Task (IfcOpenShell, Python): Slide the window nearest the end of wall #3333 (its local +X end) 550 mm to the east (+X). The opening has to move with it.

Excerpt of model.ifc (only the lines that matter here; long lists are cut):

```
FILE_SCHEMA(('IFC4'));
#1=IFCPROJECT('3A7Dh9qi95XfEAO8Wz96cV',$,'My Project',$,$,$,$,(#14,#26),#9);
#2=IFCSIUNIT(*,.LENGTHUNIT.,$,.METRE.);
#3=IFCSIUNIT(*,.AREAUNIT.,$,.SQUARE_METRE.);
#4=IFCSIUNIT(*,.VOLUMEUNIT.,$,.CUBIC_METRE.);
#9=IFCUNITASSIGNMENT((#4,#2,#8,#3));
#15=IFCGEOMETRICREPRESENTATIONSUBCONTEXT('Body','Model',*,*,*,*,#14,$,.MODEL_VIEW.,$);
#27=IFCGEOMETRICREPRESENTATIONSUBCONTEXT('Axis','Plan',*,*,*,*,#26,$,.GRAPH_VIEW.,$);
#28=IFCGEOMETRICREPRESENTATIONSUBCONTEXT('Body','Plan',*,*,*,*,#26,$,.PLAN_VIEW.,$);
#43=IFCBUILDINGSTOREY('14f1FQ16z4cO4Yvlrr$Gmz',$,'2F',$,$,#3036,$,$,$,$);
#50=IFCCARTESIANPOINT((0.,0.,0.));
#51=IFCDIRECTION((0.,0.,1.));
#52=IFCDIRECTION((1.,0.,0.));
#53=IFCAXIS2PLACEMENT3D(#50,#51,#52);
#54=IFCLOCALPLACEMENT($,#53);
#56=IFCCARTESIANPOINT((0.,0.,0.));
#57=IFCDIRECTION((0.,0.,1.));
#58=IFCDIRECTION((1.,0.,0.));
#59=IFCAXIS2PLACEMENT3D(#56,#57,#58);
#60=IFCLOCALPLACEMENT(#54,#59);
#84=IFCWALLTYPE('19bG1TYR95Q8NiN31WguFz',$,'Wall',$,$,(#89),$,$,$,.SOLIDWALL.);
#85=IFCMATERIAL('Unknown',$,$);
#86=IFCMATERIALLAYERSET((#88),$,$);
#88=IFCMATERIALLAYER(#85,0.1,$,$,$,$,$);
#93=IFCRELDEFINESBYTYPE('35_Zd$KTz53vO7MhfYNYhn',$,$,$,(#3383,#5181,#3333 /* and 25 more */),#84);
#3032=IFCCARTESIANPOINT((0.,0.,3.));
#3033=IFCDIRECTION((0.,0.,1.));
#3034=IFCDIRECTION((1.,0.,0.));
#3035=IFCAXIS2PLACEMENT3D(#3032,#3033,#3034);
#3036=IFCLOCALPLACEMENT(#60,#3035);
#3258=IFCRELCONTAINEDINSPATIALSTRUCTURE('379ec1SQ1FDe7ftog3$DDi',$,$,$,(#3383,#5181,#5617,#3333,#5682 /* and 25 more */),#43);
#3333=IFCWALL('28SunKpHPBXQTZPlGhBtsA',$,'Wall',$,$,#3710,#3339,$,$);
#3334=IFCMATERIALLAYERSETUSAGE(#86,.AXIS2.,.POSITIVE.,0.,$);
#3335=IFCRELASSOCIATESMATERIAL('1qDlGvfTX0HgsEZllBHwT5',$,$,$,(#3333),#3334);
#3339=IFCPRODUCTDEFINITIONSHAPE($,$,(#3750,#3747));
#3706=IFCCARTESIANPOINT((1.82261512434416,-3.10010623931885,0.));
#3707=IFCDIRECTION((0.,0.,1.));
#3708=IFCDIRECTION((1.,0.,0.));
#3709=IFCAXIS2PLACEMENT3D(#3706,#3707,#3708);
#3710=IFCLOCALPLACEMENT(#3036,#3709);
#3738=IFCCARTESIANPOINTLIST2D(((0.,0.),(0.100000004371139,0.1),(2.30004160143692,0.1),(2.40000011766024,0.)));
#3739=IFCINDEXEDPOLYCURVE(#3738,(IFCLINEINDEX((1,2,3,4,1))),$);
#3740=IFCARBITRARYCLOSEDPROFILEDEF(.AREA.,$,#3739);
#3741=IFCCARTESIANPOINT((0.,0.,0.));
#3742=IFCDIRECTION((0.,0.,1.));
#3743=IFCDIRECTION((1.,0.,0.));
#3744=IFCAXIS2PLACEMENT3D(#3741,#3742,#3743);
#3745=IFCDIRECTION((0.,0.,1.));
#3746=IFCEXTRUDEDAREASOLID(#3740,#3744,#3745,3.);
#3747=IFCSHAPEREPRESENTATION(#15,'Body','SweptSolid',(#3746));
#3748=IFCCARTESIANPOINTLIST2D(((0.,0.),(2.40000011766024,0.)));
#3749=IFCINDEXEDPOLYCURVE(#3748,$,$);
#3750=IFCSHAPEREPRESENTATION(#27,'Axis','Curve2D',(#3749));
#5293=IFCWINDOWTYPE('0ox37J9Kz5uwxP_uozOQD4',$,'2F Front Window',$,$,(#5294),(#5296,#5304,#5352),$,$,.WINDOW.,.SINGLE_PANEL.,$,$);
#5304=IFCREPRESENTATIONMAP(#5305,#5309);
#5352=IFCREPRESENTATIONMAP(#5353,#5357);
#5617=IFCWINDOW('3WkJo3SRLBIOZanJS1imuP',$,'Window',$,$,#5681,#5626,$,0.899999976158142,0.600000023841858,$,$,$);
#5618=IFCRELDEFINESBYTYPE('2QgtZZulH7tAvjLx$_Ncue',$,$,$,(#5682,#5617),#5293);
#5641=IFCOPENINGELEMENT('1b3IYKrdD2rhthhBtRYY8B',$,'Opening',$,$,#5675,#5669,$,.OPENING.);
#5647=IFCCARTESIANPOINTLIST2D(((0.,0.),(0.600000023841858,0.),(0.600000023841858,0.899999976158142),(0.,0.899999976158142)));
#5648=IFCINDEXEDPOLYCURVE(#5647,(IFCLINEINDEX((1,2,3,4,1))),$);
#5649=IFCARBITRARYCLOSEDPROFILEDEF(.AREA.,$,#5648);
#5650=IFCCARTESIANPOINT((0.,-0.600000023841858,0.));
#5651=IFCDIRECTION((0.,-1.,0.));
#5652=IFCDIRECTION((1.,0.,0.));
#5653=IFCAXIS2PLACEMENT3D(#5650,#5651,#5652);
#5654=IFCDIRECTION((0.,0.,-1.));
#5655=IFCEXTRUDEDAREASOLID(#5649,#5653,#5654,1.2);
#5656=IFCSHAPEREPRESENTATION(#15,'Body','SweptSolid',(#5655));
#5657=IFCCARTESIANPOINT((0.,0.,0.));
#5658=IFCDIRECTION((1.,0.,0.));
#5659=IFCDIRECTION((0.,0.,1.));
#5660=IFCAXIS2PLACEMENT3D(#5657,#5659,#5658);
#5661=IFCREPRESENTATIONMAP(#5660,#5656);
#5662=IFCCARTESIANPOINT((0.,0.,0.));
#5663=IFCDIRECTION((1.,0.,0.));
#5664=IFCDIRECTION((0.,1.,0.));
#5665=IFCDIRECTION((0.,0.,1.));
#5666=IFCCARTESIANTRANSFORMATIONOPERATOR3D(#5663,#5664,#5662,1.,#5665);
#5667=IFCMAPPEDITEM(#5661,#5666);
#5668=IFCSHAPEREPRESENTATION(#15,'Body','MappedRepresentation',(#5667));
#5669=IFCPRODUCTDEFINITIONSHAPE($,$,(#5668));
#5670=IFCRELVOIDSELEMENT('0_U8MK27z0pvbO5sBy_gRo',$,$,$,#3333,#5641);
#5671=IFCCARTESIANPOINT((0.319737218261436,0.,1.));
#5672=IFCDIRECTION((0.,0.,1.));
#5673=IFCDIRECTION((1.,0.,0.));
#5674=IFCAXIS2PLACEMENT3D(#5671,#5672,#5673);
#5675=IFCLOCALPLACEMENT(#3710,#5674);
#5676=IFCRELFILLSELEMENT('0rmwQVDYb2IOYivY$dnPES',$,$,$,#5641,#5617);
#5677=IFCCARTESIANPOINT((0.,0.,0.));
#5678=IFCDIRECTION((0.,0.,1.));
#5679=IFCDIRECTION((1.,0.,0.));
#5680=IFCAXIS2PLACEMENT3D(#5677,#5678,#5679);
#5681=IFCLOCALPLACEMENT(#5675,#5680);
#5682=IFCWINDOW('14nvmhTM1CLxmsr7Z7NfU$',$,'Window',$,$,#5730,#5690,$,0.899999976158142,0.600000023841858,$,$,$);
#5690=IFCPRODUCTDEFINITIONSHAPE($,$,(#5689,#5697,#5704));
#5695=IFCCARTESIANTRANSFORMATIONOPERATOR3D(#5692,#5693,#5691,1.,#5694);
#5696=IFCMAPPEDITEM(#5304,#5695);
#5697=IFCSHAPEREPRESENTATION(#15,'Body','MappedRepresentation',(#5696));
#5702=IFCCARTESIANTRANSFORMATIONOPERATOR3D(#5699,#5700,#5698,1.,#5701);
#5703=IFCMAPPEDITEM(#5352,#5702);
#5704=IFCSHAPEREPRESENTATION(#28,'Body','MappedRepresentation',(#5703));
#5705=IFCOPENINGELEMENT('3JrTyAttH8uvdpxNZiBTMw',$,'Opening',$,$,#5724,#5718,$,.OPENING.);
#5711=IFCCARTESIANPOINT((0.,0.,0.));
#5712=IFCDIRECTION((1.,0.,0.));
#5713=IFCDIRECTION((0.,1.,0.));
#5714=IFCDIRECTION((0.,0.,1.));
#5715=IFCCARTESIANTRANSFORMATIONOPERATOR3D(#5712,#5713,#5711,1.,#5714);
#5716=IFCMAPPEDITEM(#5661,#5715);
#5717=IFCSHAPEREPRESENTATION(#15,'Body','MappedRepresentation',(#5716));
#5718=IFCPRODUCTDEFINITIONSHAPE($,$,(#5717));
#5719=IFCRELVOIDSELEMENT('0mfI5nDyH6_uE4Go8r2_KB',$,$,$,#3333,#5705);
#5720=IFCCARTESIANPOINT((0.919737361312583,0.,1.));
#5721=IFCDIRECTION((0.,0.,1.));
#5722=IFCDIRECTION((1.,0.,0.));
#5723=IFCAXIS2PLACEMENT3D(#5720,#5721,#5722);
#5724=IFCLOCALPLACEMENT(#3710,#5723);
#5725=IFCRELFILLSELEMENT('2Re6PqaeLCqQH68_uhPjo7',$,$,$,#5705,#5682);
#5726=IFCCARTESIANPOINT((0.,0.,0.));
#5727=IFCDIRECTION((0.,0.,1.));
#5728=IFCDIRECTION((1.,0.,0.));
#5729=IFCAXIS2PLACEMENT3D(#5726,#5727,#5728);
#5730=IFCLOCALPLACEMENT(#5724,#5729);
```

```python
import ifcopenshell
import ifcopenshell.api.geometry
import ifcopenshell.util.placement
import ifcopenshell.util.unit

model = ifcopenshell.open("model.ifc")
unit_scale = ifcopenshell.util.unit.calculate_unit_scale(model)

window = model.by_guid("14nvmhTM1CLxmsr7Z7NfU$")
opening = window.FillsVoids[0].RelatingOpeningElement
wall = opening.VoidsElements[0].RelatingBuildingElement

wall_matrix = ifcopenshell.util.placement.get_local_placement(wall.ObjectPlacement)
shift = wall_matrix[:3, 0] * 0.55 / unit_scale
before = ifcopenshell.util.placement.get_local_placement(window.ObjectPlacement)[:3, 3].copy()

# The window is placed relative to its opening, so it follows when the opening moves.
matrix = ifcopenshell.util.placement.get_local_placement(opening.ObjectPlacement)
matrix[:3, 3] += shift
ifcopenshell.api.geometry.edit_object_placement(
    model, product=opening, matrix=matrix, is_si=False, should_transform_children=True
)

after = ifcopenshell.util.placement.get_local_placement(window.ObjectPlacement)[:3, 3]
print("window moved by", (after - before).round(3) + 0.0)

model.write("model_updated.ifc")
```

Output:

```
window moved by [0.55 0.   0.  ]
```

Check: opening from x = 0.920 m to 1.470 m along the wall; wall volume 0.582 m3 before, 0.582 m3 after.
